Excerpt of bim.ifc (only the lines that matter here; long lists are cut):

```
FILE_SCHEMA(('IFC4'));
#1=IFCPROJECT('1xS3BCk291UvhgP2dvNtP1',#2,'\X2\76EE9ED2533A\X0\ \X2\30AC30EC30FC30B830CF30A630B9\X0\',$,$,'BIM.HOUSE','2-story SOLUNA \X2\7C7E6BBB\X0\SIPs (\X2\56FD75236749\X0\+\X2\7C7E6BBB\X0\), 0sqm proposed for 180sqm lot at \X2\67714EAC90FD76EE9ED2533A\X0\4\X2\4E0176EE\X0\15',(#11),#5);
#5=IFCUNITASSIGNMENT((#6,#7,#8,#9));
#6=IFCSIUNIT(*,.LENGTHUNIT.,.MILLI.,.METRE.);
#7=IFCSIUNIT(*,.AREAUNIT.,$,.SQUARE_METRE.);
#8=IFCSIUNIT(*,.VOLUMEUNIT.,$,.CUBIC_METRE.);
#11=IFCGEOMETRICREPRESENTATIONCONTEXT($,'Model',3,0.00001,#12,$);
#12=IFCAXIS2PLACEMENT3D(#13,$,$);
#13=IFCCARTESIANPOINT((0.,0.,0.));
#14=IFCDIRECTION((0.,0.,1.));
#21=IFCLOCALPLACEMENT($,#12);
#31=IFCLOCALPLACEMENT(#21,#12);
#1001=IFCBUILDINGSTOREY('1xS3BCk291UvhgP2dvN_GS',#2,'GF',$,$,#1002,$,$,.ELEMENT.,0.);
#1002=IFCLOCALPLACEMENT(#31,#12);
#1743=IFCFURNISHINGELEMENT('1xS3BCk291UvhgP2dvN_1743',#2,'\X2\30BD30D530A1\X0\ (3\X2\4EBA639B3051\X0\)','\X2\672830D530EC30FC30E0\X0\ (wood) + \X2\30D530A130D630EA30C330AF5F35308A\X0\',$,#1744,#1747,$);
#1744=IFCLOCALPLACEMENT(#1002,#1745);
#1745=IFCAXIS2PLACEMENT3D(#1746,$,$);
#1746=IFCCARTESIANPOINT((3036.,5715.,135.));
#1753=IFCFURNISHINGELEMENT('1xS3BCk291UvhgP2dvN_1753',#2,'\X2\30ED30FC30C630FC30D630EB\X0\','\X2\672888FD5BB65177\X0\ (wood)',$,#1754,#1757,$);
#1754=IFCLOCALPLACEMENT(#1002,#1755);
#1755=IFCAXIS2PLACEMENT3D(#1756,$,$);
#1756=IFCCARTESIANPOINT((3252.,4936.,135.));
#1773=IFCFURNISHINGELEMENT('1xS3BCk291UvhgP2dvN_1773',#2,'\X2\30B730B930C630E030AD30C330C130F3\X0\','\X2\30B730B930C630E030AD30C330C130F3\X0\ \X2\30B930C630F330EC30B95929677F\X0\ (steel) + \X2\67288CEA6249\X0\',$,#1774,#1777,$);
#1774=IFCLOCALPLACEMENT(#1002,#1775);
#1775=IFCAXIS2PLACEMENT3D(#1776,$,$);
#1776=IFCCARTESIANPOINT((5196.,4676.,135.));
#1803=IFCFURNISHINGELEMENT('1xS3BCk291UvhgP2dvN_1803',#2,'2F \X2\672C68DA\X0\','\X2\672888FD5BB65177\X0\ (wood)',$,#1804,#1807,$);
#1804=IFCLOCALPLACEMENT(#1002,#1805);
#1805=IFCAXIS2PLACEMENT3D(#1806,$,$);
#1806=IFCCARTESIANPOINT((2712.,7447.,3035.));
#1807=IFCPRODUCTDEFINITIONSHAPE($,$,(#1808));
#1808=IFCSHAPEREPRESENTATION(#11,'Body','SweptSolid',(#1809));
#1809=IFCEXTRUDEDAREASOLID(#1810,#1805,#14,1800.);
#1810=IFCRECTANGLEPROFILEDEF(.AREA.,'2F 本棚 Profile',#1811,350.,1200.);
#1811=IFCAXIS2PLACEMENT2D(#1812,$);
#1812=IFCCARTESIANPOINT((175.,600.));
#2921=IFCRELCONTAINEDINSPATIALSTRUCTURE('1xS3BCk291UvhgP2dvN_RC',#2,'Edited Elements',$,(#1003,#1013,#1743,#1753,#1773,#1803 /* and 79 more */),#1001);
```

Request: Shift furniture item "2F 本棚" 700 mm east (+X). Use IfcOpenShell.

```python
import ifcopenshell
import ifcopenshell.api.geometry
import ifcopenshell.util.placement
import ifcopenshell.util.unit

model = ifcopenshell.open("bim.ifc")
unit_scale = ifcopenshell.util.unit.calculate_unit_scale(model)

item = model.by_guid("1xS3BCk291UvhgP2dvN_1803")
matrix = ifcopenshell.util.placement.get_local_placement(item.ObjectPlacement)
matrix[0, 3] += 0.7 / unit_scale
ifcopenshell.api.geometry.edit_object_placement(model, product=item, matrix=matrix, is_si=False)

print(ifcopenshell.util.placement.get_local_placement(item.ObjectPlacement).round(3) + 0.0)

model.write("bim_v2.ifc")
```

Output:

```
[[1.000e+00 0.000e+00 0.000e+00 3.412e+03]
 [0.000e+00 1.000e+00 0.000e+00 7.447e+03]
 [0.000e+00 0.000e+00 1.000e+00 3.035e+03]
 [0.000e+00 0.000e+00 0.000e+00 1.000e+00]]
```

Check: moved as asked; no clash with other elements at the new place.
